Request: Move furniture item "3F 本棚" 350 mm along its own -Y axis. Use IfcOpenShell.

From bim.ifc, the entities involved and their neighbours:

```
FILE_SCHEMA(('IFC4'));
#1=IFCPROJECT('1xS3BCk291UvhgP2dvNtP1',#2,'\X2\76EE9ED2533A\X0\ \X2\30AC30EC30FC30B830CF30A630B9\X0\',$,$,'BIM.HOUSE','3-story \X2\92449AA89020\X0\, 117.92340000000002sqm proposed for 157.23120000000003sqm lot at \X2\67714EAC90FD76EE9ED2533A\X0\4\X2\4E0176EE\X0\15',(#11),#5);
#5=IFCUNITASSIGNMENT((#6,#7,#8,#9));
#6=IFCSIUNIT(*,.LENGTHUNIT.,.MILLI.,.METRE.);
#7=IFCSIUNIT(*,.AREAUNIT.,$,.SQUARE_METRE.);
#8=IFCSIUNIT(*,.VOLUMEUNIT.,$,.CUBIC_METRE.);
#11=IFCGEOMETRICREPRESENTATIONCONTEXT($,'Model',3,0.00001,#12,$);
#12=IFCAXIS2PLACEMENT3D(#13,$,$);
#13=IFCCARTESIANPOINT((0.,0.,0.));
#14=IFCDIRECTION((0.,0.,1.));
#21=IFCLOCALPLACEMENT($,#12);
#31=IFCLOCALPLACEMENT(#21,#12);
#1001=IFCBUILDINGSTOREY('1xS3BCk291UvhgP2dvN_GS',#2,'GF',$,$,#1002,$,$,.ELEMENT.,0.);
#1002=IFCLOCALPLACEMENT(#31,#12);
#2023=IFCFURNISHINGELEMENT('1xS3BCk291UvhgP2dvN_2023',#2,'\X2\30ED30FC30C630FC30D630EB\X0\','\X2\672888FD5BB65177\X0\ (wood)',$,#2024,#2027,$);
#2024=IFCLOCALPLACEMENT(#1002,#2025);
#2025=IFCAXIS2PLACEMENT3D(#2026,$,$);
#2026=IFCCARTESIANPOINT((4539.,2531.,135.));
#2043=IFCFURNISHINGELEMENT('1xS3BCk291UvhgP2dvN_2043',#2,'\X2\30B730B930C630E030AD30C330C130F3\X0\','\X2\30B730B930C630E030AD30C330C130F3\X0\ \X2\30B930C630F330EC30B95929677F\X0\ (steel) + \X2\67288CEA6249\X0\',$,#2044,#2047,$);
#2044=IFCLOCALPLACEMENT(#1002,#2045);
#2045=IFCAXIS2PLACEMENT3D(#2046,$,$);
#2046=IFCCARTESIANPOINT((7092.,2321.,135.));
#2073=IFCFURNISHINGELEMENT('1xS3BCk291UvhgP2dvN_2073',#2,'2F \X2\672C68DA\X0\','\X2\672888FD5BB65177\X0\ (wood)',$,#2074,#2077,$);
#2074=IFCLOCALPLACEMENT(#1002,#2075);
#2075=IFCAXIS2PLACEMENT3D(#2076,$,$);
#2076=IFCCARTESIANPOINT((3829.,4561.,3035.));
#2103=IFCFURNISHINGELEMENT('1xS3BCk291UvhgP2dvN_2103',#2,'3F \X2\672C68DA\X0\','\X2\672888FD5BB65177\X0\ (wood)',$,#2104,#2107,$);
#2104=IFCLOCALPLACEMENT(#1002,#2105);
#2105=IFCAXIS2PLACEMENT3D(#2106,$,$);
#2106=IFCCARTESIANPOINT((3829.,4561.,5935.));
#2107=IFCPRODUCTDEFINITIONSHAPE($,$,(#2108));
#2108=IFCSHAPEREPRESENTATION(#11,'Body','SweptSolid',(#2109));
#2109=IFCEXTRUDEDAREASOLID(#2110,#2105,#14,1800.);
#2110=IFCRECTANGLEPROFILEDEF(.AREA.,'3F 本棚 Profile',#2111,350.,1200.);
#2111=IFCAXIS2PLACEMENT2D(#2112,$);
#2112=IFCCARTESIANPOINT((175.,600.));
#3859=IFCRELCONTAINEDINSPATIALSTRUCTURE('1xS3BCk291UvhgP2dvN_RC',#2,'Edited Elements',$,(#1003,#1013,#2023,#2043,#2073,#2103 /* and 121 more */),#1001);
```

```python
import ifcopenshell
import ifcopenshell.api.geometry
import ifcopenshell.util.placement
import ifcopenshell.util.unit

model = ifcopenshell.open("bim.ifc")
unit_scale = ifcopenshell.util.unit.calculate_unit_scale(model)

item = model.by_guid("1xS3BCk291UvhgP2dvN_2103")
matrix = ifcopenshell.util.placement.get_local_placement(item.ObjectPlacement)
matrix[:3, 3] -= matrix[:3, 1] * 0.35 / unit_scale
ifcopenshell.api.geometry.edit_object_placement(model, product=item, matrix=matrix, is_si=False)

print(ifcopenshell.util.placement.get_local_placement(item.ObjectPlacement).round(3) + 0.0)

model.write("bim_edited.ifc")
```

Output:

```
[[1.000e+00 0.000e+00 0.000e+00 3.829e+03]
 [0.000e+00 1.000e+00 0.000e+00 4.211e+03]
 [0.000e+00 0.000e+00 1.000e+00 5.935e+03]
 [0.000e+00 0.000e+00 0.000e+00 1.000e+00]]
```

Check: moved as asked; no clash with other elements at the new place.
